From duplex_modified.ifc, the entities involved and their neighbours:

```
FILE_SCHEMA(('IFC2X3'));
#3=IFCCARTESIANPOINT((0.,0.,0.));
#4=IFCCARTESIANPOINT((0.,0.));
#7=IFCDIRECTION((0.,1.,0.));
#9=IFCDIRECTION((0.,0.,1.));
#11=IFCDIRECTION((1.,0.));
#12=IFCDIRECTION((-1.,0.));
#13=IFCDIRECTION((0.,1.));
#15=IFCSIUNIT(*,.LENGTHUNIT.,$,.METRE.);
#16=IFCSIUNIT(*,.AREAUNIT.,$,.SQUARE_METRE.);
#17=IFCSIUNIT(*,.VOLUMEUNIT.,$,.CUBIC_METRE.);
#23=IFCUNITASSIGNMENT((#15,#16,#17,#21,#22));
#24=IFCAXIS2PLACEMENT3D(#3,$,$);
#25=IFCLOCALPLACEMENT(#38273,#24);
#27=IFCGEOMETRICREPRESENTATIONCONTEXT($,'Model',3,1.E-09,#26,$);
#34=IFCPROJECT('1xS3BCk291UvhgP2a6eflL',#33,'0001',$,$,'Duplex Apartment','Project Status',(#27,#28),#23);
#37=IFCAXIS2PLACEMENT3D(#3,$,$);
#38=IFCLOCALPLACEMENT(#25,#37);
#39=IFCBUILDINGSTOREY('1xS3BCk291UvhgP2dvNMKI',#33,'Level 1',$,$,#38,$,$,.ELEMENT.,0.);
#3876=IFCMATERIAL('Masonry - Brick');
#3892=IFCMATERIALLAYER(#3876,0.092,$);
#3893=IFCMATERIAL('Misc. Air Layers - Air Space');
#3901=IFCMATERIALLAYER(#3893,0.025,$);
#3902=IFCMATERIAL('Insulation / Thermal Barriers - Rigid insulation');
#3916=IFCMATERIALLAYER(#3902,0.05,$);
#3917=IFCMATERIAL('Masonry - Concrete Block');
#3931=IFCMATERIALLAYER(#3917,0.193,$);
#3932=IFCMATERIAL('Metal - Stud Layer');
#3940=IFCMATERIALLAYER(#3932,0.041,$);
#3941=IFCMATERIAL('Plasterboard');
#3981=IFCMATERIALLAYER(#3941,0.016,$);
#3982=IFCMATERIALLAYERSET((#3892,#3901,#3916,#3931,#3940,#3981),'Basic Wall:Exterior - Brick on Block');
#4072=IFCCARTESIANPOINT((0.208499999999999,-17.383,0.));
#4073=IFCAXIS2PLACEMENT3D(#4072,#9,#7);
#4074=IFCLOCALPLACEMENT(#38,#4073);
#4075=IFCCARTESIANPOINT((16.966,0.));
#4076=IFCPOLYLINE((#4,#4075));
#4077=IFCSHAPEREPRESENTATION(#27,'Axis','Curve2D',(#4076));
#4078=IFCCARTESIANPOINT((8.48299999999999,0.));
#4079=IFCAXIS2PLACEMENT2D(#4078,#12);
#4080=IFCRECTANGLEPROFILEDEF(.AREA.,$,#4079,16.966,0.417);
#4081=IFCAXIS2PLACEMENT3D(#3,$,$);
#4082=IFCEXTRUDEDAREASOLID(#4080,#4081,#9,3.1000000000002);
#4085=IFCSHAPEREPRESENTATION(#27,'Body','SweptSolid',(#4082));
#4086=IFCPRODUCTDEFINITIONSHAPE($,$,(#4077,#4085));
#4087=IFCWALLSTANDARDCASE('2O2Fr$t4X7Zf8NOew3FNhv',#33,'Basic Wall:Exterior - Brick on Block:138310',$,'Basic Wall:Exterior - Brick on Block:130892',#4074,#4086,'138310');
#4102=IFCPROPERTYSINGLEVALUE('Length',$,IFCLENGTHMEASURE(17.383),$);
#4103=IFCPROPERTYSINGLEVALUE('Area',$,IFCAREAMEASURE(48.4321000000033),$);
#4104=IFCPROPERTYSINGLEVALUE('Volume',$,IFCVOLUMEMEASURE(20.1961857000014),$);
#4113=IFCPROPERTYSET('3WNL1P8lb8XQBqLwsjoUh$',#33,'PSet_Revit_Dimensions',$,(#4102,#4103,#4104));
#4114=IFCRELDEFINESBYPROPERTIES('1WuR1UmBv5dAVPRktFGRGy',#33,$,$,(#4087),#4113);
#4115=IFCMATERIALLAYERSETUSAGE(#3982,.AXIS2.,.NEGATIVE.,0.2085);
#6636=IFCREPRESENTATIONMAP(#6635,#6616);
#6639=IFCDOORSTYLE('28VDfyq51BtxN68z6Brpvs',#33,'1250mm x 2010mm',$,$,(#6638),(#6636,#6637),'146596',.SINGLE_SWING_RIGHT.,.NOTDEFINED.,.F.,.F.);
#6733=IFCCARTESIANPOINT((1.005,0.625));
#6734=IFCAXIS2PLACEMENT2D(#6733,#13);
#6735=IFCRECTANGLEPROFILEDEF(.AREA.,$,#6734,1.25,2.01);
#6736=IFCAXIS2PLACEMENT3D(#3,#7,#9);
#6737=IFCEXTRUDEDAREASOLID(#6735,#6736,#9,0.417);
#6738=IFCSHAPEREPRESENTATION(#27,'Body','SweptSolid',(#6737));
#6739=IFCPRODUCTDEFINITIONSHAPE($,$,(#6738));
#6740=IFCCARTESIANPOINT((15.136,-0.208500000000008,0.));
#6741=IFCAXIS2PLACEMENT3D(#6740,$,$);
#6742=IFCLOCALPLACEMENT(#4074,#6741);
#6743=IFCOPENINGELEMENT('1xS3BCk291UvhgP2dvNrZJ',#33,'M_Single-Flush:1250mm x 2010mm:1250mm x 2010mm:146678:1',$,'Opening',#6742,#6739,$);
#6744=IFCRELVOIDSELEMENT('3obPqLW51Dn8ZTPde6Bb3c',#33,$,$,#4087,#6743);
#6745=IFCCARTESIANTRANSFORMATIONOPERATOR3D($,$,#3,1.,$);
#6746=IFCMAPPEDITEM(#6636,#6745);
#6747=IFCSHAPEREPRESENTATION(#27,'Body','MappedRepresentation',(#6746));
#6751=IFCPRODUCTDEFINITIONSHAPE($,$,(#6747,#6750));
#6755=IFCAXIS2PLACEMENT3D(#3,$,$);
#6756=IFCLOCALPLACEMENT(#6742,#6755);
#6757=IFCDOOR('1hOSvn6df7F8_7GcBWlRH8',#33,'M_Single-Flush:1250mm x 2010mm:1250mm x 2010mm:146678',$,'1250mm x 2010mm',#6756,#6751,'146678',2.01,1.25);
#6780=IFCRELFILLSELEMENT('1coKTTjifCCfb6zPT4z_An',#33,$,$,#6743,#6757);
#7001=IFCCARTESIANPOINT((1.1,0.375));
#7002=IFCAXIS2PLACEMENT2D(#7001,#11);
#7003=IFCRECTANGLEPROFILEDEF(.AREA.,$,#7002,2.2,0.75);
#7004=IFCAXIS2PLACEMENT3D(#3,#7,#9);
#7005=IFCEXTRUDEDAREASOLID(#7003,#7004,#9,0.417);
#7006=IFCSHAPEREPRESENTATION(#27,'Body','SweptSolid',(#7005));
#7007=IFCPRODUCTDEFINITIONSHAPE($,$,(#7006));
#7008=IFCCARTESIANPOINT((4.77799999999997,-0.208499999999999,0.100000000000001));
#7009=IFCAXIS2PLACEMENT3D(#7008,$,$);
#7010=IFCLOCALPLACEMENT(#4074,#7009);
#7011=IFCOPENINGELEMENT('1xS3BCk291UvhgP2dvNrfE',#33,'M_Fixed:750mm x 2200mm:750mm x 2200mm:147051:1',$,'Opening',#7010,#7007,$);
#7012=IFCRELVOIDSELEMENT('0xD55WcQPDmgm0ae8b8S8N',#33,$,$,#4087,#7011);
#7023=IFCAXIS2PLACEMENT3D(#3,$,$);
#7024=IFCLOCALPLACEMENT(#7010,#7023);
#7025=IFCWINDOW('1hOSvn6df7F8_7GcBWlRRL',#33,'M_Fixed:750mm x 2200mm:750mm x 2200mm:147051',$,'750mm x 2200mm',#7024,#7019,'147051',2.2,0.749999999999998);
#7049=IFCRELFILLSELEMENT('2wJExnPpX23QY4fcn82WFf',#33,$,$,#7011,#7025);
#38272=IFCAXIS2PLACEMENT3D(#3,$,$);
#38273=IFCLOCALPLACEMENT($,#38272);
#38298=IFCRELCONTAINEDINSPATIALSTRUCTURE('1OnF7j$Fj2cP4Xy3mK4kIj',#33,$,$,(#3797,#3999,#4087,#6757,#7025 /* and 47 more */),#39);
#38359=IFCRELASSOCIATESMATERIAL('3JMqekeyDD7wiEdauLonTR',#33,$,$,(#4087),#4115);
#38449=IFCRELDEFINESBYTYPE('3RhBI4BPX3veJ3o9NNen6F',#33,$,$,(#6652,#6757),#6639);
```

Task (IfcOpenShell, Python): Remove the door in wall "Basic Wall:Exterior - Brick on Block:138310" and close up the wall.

```python
import ifcopenshell
import ifcopenshell.api.feature
import ifcopenshell.api.pset
import ifcopenshell.api.root
import ifcopenshell.geom
import ifcopenshell.util.element
import ifcopenshell.util.shape
import ifcopenshell.util.unit

model = ifcopenshell.open("duplex_modified.ifc")
area_scale = ifcopenshell.util.unit.calculate_unit_scale(model, "AREAUNIT")
volume_scale = ifcopenshell.util.unit.calculate_unit_scale(model, "VOLUMEUNIT")
settings = ifcopenshell.geom.settings()


def volume(element):
    """Net volume in cubic metres, openings subtracted."""
    shape = ifcopenshell.geom.create_shape(settings, element)
    return ifcopenshell.util.shape.get_volume(shape.geometry)


door = model.by_guid("1hOSvn6df7F8_7GcBWlRH8")
opening = door.FillsVoids[0].RelatingOpeningElement
wall = opening.VoidsElements[0].RelatingBuildingElement
before = volume(wall)

ifcopenshell.api.root.remove_product(model, product=door)
ifcopenshell.api.feature.remove_feature(model, feature=opening)

after = volume(wall)
thickness = 0.417  # wall thickness in metres

# Update the wall's stored quantities.
pset = model.by_id(ifcopenshell.util.element.get_pset(wall, "PSet_Revit_Dimensions", should_inherit=False)["id"])
ifcopenshell.api.pset.edit_pset(model, pset=pset, properties={
    "Area": model.create_entity("IfcAreaMeasure", after / thickness / area_scale),
    "Volume": model.create_entity("IfcVolumeMeasure", after / volume_scale),
})

print(f"wall volume {before:.3f} -> {after:.3f} m3")

model.write("duplex_modified_updated.ifc")
```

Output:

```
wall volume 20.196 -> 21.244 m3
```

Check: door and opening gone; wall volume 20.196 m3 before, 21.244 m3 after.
